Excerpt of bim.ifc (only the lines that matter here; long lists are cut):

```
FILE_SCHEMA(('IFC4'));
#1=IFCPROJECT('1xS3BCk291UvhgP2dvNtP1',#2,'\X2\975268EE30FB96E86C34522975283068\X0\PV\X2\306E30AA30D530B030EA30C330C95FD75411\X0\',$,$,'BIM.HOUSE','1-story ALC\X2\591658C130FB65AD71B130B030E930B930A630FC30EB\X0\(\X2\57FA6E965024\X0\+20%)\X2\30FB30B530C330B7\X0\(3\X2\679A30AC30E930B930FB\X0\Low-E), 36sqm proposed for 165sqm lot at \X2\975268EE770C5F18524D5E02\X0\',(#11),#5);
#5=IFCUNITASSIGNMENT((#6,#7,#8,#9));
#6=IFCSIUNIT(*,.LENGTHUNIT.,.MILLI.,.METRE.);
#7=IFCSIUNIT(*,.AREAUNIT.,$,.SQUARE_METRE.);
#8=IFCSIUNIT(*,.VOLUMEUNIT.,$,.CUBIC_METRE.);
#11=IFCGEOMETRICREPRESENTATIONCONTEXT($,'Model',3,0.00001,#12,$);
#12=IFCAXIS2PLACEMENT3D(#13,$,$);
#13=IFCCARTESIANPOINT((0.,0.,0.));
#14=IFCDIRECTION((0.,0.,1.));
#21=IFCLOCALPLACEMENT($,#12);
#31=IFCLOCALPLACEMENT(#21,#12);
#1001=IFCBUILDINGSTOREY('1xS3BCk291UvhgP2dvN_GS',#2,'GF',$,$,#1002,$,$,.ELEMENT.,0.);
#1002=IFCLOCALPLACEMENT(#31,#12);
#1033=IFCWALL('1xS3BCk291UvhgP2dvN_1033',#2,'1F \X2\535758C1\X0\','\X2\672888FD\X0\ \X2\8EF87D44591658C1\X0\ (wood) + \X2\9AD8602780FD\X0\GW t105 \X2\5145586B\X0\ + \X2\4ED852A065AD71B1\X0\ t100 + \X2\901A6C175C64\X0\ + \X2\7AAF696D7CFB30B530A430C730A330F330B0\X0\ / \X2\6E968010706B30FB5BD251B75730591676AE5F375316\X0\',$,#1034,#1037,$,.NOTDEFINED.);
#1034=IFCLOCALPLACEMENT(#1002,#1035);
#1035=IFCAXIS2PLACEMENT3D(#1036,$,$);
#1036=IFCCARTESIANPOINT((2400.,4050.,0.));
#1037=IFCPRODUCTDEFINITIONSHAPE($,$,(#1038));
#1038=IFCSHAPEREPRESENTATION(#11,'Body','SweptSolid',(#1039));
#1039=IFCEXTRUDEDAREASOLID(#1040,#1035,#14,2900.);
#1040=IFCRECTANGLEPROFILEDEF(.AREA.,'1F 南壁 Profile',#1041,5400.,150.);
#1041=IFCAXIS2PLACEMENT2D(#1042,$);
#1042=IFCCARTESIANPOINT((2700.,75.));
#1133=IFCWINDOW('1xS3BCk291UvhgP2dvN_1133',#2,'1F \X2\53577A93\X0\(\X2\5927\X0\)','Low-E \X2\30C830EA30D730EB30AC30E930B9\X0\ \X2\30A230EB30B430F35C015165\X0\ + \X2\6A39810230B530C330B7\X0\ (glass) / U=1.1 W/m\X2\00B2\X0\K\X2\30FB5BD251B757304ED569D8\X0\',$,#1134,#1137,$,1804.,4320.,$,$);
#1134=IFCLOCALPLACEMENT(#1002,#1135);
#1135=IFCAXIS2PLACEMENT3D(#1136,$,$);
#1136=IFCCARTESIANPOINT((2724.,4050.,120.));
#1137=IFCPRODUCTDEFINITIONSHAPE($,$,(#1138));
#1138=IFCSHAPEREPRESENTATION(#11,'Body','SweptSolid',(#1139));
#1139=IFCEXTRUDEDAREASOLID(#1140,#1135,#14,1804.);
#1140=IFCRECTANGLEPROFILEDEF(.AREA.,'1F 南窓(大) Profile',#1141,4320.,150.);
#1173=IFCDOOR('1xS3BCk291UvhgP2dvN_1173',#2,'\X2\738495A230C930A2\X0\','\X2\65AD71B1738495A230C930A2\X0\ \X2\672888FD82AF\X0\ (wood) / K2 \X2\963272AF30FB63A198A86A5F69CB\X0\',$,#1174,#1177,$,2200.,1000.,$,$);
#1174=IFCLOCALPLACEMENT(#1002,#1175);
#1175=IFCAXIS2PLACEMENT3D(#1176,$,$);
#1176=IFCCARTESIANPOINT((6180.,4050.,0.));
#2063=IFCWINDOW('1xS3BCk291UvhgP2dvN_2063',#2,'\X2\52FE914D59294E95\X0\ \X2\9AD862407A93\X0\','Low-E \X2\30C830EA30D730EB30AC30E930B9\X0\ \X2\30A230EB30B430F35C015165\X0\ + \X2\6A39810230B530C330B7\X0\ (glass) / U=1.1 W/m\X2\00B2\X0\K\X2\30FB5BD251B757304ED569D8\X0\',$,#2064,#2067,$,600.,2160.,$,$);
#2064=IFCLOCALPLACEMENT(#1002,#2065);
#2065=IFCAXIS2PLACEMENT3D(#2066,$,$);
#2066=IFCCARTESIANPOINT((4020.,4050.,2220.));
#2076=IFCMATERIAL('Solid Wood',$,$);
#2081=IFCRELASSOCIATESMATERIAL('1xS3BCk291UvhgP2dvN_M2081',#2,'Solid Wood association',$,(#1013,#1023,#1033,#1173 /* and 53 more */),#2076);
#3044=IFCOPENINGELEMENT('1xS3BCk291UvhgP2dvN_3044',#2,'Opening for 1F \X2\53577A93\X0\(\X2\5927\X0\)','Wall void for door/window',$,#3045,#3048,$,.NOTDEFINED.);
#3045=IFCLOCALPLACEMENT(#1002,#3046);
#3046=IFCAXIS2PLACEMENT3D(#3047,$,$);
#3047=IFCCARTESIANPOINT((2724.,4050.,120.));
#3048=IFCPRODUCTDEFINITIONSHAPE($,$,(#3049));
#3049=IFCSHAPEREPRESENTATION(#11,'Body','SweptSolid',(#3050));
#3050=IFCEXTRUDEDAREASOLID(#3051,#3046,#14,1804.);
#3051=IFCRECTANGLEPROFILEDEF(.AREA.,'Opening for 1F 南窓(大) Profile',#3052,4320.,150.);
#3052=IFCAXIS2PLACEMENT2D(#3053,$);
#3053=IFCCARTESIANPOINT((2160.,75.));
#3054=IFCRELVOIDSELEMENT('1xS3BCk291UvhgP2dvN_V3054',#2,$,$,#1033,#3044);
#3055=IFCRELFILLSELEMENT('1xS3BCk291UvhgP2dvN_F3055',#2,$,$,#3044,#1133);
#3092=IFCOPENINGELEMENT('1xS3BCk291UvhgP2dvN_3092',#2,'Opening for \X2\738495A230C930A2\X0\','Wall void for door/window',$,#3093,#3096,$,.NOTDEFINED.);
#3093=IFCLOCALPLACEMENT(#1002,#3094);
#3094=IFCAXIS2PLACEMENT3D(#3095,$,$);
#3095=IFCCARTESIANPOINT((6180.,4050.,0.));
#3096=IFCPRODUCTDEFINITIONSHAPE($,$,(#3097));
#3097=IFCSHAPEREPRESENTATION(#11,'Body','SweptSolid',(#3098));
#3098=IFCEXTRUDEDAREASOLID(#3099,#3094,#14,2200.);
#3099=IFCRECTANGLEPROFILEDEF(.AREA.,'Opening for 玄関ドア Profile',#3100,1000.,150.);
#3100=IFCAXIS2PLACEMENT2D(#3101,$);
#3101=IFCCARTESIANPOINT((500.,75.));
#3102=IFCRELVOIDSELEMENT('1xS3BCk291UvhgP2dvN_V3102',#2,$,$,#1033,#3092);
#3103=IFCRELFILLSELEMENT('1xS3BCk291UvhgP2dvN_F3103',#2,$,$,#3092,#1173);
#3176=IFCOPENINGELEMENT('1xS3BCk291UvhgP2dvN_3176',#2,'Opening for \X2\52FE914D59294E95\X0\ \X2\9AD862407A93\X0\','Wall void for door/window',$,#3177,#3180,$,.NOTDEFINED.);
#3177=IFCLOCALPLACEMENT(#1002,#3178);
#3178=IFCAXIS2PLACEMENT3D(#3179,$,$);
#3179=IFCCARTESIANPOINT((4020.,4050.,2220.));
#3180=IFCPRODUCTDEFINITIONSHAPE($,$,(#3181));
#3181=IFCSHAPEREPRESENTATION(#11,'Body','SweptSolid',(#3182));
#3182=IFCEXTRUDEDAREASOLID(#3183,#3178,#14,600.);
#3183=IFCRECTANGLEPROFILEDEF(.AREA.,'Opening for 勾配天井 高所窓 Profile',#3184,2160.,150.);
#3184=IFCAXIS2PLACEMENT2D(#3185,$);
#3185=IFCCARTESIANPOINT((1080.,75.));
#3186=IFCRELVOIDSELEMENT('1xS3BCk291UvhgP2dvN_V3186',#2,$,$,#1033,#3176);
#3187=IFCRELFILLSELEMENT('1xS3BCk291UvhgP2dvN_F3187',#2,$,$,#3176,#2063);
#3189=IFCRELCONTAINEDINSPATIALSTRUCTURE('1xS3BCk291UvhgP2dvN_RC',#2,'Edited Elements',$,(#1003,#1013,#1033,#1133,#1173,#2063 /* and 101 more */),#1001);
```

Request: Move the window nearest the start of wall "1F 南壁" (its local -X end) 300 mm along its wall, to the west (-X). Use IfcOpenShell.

```python
import ifcopenshell
import ifcopenshell.api.geometry
import ifcopenshell.util.placement
import ifcopenshell.util.unit

model = ifcopenshell.open("bim.ifc")
unit_scale = ifcopenshell.util.unit.calculate_unit_scale(model)

window = model.by_guid("1xS3BCk291UvhgP2dvN_1133")
opening = window.FillsVoids[0].RelatingOpeningElement
wall = opening.VoidsElements[0].RelatingBuildingElement

wall_matrix = ifcopenshell.util.placement.get_local_placement(wall.ObjectPlacement)
shift = wall_matrix[:3, 0] * -0.3 / unit_scale
before = ifcopenshell.util.placement.get_local_placement(window.ObjectPlacement)[:3, 3].copy()

# The window is not placed relative to its opening, so move both.
for product in (opening, window):
    matrix = ifcopenshell.util.placement.get_local_placement(product.ObjectPlacement)
    matrix[:3, 3] += shift
    ifcopenshell.api.geometry.edit_object_placement(model, product=product, matrix=matrix, is_si=False)

after = ifcopenshell.util.placement.get_local_placement(window.ObjectPlacement)[:3, 3]
print("window moved by", (after - before).round(3) + 0.0)

model.write("bim_v2.ifc")
```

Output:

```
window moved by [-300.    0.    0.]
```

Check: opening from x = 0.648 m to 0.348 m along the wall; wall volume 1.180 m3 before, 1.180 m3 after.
